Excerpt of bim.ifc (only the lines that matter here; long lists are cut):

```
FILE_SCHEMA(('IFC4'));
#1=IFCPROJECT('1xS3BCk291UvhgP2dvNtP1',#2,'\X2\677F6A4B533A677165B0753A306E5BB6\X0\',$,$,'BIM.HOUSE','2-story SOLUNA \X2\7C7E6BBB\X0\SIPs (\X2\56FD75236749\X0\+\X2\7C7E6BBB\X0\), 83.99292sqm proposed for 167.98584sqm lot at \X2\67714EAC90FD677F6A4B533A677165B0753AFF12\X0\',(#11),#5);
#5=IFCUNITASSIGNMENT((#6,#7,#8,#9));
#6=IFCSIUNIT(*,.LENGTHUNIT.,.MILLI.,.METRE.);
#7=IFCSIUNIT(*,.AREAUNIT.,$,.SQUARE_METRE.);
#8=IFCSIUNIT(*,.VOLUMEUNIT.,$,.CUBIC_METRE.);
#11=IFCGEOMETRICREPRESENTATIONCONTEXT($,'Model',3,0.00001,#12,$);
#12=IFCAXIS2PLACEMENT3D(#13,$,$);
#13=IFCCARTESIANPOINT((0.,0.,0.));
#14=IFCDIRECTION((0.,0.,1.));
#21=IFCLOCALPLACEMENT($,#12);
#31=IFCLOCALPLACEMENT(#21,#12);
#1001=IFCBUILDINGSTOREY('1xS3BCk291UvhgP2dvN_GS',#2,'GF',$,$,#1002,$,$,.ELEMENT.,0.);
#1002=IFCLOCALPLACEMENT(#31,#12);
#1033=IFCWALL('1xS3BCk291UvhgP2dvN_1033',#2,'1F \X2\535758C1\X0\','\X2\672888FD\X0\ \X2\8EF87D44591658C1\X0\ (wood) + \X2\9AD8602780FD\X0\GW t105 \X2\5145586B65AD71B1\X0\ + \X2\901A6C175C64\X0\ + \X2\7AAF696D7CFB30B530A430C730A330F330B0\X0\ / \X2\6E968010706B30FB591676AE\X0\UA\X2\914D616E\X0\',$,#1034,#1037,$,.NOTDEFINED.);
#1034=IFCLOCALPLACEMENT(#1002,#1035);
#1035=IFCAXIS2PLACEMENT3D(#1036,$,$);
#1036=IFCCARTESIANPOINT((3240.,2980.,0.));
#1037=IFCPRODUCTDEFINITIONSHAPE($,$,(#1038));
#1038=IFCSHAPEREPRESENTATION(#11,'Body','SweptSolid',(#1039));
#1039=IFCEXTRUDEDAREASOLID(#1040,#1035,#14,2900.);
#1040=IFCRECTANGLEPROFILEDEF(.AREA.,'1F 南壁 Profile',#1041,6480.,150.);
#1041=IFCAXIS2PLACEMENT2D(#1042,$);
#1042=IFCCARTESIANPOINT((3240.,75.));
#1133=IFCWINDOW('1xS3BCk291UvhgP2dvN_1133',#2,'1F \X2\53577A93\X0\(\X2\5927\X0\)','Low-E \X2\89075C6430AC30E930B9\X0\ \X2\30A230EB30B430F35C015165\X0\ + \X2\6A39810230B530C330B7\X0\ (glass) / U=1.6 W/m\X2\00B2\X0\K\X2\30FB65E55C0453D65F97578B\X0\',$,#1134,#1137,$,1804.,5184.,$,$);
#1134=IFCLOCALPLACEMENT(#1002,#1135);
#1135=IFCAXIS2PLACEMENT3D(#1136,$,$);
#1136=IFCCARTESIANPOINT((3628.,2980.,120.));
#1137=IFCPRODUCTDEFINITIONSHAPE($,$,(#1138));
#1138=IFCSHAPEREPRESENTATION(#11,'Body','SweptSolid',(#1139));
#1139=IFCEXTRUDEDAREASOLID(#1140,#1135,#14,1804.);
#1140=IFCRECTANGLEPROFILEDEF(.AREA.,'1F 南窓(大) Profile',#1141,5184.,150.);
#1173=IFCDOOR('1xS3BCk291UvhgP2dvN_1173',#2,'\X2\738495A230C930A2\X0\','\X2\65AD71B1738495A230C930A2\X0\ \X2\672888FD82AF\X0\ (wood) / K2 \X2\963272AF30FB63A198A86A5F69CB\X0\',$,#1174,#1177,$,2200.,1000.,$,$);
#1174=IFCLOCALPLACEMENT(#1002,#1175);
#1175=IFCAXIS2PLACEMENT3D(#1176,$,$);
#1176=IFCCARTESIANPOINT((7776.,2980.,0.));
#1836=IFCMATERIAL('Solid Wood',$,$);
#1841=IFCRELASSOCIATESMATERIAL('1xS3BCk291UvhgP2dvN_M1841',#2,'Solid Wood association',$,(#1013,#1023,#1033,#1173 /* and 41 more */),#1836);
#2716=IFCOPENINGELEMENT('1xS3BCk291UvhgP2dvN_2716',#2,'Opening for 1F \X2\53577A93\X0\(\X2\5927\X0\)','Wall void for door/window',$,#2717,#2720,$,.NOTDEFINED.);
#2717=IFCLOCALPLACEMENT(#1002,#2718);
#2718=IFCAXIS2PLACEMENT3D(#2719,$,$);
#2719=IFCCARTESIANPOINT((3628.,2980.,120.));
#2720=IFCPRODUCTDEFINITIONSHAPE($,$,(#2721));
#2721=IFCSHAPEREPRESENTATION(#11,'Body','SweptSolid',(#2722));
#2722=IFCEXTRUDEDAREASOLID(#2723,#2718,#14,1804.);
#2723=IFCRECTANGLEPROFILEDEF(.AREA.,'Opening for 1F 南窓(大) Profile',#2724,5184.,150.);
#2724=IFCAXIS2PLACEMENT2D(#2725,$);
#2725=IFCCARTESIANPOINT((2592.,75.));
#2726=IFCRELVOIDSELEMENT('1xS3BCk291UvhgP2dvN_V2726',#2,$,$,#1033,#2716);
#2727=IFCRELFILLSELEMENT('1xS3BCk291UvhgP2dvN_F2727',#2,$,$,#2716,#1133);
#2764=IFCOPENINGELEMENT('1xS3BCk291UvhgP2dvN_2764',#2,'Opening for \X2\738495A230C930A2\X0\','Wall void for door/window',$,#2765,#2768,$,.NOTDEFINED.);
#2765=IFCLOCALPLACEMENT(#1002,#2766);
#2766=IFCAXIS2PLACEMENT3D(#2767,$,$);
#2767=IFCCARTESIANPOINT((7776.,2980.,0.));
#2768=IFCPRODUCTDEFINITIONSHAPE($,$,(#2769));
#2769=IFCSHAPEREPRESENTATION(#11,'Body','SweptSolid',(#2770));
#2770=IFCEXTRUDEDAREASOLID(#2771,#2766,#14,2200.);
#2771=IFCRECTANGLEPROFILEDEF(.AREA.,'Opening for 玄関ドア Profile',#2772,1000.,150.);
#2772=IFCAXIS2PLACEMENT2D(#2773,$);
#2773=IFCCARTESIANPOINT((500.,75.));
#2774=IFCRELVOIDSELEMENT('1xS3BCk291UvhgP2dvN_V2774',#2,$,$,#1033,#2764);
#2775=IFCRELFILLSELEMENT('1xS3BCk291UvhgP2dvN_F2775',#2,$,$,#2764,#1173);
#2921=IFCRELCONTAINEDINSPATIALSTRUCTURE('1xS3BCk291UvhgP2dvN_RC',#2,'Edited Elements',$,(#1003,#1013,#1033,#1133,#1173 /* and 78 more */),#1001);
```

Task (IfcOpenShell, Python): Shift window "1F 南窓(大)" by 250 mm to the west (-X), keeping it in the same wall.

```python
import ifcopenshell
import ifcopenshell.api.geometry
import ifcopenshell.util.placement
import ifcopenshell.util.unit

model = ifcopenshell.open("bim.ifc")
unit_scale = ifcopenshell.util.unit.calculate_unit_scale(model)

window = model.by_guid("1xS3BCk291UvhgP2dvN_1133")
opening = window.FillsVoids[0].RelatingOpeningElement
wall = opening.VoidsElements[0].RelatingBuildingElement

wall_matrix = ifcopenshell.util.placement.get_local_placement(wall.ObjectPlacement)
shift = wall_matrix[:3, 0] * -0.25 / unit_scale
before = ifcopenshell.util.placement.get_local_placement(window.ObjectPlacement)[:3, 3].copy()

# The window is not placed relative to its opening, so move both.
for product in (opening, window):
    matrix = ifcopenshell.util.placement.get_local_placement(product.ObjectPlacement)
    matrix[:3, 3] += shift
    ifcopenshell.api.geometry.edit_object_placement(model, product=product, matrix=matrix, is_si=False)

after = ifcopenshell.util.placement.get_local_placement(window.ObjectPlacement)[:3, 3]
print("window moved by", (after - before).round(3) + 0.0)

model.write("bim_rev.ifc")
```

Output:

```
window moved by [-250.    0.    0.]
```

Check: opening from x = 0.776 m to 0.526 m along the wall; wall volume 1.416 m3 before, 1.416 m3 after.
